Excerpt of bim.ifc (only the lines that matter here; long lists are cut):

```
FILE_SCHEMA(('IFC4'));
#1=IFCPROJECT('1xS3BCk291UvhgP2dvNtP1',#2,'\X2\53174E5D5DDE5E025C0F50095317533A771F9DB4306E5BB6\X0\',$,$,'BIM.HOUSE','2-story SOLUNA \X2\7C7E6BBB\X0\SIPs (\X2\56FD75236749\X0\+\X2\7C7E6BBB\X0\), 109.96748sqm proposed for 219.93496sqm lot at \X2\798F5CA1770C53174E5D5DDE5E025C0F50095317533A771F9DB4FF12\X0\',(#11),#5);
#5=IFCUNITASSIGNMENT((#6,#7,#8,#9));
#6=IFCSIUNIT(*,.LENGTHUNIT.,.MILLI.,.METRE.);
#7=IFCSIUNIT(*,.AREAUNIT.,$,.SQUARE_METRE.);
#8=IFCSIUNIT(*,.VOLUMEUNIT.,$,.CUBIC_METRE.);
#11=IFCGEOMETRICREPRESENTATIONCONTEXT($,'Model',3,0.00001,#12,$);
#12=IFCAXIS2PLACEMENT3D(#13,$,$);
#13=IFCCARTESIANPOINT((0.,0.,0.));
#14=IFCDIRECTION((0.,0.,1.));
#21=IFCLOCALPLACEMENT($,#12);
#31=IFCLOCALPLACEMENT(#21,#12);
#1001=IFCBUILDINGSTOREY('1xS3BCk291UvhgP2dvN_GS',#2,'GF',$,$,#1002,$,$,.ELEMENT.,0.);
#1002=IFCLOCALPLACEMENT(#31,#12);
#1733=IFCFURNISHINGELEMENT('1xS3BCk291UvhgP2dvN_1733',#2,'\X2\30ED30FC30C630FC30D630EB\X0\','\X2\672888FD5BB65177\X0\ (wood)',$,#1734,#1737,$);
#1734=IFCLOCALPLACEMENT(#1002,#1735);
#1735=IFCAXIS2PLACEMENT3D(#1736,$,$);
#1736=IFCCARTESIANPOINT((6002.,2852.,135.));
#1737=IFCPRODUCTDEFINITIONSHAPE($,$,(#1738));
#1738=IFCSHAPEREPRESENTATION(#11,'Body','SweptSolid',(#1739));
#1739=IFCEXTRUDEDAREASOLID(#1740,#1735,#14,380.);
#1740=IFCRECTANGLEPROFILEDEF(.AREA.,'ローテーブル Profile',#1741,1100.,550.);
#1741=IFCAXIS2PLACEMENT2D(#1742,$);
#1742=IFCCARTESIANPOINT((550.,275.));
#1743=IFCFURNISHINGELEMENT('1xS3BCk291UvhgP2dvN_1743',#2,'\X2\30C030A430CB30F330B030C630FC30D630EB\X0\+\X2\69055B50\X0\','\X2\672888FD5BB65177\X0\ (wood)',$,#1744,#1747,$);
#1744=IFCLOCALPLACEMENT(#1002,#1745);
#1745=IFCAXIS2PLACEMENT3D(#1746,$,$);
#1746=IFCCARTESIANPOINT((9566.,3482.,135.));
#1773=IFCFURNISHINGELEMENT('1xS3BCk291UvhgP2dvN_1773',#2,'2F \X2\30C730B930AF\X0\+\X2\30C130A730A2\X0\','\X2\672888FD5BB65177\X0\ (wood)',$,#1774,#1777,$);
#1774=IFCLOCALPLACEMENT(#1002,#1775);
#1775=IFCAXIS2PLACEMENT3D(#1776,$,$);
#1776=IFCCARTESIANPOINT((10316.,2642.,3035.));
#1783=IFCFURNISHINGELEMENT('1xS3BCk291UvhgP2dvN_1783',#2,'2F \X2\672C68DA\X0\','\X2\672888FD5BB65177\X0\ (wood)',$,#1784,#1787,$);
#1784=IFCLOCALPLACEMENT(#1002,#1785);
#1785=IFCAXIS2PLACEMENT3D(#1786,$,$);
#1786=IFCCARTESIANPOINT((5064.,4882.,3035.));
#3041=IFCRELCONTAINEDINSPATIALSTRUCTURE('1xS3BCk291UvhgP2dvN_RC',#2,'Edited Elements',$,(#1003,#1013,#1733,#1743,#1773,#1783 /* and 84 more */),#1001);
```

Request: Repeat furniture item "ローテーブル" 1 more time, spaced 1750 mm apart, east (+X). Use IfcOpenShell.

```python
import numpy as np
import ifcopenshell
import ifcopenshell.api.geometry
import ifcopenshell.api.root
import ifcopenshell.util.element
import ifcopenshell.util.placement
import ifcopenshell.util.unit

model = ifcopenshell.open("bim.ifc")
unit_scale = ifcopenshell.util.unit.calculate_unit_scale(model)


def reuse_history(source, copy):
    """copy_class also copies each property set's owner history, people and application; keep the originals."""
    for rel in copy.IsDefinedBy:
        if rel.is_a("IfcRelDefinesByProperties") and (history := rel.RelatingPropertyDefinition.OwnerHistory):
            rel.RelatingPropertyDefinition.OwnerHistory = source.OwnerHistory
            ifcopenshell.util.element.remove_deep2(model, history)


source = model.by_id(1733)
base = ifcopenshell.util.placement.get_local_placement(source.ObjectPlacement)
step = np.array([1.0, 0.0, 0.0]) * 1.75 / unit_scale

for i in range(1, 2):
    copy = ifcopenshell.api.root.copy_class(model, product=source)
    copy.Representation = ifcopenshell.util.element.copy_deep(
        model, source.Representation, exclude=["IfcGeometricRepresentationContext", "IfcRepresentationMap"]
    )
    reuse_history(source, copy)
    matrix = base.copy()
    matrix[:3, 3] += i * step
    print("added at", matrix[:3, 3].round(3) + 0.0)
    ifcopenshell.api.geometry.edit_object_placement(model, product=copy, matrix=matrix, is_si=False)

model.write("bim-out.ifc")
```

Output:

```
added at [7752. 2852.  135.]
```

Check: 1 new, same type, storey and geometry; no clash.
